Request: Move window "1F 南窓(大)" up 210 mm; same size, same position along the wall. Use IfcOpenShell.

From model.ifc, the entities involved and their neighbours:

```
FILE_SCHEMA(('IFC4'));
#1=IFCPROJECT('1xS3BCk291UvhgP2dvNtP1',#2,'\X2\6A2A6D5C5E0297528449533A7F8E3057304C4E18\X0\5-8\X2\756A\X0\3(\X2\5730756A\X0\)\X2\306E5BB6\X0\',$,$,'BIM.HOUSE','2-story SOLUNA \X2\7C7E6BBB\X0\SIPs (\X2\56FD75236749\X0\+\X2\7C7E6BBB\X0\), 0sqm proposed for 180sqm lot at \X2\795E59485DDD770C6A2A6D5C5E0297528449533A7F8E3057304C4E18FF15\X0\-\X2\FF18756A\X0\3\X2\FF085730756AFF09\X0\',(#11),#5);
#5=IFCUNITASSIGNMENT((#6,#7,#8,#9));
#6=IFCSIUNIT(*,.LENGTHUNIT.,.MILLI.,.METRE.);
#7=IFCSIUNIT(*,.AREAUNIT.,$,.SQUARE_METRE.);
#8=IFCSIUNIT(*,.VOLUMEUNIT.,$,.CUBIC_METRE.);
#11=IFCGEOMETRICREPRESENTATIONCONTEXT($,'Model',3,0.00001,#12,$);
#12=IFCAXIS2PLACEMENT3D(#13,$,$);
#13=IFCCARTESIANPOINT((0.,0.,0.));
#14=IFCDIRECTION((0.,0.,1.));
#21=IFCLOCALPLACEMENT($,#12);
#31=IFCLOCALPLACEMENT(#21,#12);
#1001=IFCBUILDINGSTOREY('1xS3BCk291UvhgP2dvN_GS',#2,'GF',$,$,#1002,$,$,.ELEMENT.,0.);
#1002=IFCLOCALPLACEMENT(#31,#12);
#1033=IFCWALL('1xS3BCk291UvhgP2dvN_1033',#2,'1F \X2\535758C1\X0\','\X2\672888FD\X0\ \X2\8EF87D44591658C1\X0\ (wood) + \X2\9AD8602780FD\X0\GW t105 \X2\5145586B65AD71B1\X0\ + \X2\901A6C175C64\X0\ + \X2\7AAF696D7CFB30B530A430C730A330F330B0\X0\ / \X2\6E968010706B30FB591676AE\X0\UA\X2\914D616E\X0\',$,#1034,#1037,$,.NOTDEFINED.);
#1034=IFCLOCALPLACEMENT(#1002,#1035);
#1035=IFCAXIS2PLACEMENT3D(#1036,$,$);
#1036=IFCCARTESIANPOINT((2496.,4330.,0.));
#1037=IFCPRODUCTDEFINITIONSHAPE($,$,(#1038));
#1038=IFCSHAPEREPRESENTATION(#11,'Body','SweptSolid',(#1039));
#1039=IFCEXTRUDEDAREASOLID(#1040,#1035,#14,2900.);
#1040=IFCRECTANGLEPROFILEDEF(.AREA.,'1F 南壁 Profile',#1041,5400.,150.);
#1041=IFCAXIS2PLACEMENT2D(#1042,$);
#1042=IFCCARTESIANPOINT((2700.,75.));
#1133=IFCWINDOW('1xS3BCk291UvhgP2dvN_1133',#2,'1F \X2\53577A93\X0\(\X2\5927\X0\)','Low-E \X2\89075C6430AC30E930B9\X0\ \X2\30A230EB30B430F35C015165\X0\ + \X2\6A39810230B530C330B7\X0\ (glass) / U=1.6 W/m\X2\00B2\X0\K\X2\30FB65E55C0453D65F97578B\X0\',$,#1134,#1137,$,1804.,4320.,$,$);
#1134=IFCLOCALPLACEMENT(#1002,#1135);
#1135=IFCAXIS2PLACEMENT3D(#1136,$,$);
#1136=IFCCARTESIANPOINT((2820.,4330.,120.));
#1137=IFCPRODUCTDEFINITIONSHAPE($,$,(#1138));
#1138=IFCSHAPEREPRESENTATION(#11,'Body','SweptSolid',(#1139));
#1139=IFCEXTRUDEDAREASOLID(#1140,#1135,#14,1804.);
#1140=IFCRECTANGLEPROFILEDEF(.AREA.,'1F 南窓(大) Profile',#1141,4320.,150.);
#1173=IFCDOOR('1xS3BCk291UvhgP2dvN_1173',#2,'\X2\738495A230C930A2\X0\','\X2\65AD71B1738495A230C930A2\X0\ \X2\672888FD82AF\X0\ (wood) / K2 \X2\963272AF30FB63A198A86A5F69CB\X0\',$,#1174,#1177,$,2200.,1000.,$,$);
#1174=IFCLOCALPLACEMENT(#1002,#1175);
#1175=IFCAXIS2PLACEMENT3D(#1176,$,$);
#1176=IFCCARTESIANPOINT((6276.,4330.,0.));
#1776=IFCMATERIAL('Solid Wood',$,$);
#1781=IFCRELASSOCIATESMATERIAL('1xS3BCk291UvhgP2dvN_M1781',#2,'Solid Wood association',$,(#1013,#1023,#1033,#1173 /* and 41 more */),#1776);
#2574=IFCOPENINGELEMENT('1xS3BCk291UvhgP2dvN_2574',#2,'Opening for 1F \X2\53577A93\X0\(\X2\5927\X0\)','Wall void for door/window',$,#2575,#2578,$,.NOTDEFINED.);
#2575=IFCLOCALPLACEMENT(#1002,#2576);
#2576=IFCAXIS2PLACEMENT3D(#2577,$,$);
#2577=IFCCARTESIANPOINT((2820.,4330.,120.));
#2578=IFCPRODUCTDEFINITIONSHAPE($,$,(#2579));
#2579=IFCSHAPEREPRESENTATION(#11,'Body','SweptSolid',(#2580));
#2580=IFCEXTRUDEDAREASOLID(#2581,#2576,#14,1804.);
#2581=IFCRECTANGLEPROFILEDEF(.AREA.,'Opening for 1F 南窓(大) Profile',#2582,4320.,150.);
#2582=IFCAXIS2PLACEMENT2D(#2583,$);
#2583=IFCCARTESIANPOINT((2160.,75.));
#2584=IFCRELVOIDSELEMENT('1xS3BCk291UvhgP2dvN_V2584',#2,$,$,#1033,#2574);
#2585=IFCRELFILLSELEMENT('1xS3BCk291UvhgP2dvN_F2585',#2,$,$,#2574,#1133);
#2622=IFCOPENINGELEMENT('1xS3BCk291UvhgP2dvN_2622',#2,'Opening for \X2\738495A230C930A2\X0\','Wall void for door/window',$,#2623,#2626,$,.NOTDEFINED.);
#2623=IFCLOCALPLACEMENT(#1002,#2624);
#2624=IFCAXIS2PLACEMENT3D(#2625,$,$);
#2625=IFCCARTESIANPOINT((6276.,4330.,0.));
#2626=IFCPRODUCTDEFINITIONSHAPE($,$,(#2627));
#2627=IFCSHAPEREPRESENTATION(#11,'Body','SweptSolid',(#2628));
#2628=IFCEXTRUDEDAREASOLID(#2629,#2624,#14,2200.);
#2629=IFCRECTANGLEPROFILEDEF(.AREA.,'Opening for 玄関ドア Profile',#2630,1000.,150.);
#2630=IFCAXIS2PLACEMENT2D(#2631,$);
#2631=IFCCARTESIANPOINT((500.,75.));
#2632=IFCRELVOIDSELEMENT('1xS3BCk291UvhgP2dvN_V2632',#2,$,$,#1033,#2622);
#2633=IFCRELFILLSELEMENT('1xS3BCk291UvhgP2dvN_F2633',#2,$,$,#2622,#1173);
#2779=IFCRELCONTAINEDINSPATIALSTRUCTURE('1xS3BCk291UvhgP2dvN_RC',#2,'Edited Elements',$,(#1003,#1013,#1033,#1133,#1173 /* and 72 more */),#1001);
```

```python
import numpy as np
import ifcopenshell
import ifcopenshell.api.geometry
import ifcopenshell.util.placement
import ifcopenshell.util.unit

model = ifcopenshell.open("model.ifc")
unit_scale = ifcopenshell.util.unit.calculate_unit_scale(model)

window = model.by_guid("1xS3BCk291UvhgP2dvN_1133")
opening = window.FillsVoids[0].RelatingOpeningElement
dz = 0.21 / unit_scale

shift = np.array([0.0, 0.0, dz])
# The window is not placed relative to its opening, so move both.
for product in (opening, window):
    matrix = ifcopenshell.util.placement.get_local_placement(product.ObjectPlacement)
    matrix[:3, 3] += shift
    ifcopenshell.api.geometry.edit_object_placement(model, product=product, matrix=matrix, is_si=False)

print(f"moved by {dz * unit_scale:+.3f} m")

model.write("model_v2.ifc")
```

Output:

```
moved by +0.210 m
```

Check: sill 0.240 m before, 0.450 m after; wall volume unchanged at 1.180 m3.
